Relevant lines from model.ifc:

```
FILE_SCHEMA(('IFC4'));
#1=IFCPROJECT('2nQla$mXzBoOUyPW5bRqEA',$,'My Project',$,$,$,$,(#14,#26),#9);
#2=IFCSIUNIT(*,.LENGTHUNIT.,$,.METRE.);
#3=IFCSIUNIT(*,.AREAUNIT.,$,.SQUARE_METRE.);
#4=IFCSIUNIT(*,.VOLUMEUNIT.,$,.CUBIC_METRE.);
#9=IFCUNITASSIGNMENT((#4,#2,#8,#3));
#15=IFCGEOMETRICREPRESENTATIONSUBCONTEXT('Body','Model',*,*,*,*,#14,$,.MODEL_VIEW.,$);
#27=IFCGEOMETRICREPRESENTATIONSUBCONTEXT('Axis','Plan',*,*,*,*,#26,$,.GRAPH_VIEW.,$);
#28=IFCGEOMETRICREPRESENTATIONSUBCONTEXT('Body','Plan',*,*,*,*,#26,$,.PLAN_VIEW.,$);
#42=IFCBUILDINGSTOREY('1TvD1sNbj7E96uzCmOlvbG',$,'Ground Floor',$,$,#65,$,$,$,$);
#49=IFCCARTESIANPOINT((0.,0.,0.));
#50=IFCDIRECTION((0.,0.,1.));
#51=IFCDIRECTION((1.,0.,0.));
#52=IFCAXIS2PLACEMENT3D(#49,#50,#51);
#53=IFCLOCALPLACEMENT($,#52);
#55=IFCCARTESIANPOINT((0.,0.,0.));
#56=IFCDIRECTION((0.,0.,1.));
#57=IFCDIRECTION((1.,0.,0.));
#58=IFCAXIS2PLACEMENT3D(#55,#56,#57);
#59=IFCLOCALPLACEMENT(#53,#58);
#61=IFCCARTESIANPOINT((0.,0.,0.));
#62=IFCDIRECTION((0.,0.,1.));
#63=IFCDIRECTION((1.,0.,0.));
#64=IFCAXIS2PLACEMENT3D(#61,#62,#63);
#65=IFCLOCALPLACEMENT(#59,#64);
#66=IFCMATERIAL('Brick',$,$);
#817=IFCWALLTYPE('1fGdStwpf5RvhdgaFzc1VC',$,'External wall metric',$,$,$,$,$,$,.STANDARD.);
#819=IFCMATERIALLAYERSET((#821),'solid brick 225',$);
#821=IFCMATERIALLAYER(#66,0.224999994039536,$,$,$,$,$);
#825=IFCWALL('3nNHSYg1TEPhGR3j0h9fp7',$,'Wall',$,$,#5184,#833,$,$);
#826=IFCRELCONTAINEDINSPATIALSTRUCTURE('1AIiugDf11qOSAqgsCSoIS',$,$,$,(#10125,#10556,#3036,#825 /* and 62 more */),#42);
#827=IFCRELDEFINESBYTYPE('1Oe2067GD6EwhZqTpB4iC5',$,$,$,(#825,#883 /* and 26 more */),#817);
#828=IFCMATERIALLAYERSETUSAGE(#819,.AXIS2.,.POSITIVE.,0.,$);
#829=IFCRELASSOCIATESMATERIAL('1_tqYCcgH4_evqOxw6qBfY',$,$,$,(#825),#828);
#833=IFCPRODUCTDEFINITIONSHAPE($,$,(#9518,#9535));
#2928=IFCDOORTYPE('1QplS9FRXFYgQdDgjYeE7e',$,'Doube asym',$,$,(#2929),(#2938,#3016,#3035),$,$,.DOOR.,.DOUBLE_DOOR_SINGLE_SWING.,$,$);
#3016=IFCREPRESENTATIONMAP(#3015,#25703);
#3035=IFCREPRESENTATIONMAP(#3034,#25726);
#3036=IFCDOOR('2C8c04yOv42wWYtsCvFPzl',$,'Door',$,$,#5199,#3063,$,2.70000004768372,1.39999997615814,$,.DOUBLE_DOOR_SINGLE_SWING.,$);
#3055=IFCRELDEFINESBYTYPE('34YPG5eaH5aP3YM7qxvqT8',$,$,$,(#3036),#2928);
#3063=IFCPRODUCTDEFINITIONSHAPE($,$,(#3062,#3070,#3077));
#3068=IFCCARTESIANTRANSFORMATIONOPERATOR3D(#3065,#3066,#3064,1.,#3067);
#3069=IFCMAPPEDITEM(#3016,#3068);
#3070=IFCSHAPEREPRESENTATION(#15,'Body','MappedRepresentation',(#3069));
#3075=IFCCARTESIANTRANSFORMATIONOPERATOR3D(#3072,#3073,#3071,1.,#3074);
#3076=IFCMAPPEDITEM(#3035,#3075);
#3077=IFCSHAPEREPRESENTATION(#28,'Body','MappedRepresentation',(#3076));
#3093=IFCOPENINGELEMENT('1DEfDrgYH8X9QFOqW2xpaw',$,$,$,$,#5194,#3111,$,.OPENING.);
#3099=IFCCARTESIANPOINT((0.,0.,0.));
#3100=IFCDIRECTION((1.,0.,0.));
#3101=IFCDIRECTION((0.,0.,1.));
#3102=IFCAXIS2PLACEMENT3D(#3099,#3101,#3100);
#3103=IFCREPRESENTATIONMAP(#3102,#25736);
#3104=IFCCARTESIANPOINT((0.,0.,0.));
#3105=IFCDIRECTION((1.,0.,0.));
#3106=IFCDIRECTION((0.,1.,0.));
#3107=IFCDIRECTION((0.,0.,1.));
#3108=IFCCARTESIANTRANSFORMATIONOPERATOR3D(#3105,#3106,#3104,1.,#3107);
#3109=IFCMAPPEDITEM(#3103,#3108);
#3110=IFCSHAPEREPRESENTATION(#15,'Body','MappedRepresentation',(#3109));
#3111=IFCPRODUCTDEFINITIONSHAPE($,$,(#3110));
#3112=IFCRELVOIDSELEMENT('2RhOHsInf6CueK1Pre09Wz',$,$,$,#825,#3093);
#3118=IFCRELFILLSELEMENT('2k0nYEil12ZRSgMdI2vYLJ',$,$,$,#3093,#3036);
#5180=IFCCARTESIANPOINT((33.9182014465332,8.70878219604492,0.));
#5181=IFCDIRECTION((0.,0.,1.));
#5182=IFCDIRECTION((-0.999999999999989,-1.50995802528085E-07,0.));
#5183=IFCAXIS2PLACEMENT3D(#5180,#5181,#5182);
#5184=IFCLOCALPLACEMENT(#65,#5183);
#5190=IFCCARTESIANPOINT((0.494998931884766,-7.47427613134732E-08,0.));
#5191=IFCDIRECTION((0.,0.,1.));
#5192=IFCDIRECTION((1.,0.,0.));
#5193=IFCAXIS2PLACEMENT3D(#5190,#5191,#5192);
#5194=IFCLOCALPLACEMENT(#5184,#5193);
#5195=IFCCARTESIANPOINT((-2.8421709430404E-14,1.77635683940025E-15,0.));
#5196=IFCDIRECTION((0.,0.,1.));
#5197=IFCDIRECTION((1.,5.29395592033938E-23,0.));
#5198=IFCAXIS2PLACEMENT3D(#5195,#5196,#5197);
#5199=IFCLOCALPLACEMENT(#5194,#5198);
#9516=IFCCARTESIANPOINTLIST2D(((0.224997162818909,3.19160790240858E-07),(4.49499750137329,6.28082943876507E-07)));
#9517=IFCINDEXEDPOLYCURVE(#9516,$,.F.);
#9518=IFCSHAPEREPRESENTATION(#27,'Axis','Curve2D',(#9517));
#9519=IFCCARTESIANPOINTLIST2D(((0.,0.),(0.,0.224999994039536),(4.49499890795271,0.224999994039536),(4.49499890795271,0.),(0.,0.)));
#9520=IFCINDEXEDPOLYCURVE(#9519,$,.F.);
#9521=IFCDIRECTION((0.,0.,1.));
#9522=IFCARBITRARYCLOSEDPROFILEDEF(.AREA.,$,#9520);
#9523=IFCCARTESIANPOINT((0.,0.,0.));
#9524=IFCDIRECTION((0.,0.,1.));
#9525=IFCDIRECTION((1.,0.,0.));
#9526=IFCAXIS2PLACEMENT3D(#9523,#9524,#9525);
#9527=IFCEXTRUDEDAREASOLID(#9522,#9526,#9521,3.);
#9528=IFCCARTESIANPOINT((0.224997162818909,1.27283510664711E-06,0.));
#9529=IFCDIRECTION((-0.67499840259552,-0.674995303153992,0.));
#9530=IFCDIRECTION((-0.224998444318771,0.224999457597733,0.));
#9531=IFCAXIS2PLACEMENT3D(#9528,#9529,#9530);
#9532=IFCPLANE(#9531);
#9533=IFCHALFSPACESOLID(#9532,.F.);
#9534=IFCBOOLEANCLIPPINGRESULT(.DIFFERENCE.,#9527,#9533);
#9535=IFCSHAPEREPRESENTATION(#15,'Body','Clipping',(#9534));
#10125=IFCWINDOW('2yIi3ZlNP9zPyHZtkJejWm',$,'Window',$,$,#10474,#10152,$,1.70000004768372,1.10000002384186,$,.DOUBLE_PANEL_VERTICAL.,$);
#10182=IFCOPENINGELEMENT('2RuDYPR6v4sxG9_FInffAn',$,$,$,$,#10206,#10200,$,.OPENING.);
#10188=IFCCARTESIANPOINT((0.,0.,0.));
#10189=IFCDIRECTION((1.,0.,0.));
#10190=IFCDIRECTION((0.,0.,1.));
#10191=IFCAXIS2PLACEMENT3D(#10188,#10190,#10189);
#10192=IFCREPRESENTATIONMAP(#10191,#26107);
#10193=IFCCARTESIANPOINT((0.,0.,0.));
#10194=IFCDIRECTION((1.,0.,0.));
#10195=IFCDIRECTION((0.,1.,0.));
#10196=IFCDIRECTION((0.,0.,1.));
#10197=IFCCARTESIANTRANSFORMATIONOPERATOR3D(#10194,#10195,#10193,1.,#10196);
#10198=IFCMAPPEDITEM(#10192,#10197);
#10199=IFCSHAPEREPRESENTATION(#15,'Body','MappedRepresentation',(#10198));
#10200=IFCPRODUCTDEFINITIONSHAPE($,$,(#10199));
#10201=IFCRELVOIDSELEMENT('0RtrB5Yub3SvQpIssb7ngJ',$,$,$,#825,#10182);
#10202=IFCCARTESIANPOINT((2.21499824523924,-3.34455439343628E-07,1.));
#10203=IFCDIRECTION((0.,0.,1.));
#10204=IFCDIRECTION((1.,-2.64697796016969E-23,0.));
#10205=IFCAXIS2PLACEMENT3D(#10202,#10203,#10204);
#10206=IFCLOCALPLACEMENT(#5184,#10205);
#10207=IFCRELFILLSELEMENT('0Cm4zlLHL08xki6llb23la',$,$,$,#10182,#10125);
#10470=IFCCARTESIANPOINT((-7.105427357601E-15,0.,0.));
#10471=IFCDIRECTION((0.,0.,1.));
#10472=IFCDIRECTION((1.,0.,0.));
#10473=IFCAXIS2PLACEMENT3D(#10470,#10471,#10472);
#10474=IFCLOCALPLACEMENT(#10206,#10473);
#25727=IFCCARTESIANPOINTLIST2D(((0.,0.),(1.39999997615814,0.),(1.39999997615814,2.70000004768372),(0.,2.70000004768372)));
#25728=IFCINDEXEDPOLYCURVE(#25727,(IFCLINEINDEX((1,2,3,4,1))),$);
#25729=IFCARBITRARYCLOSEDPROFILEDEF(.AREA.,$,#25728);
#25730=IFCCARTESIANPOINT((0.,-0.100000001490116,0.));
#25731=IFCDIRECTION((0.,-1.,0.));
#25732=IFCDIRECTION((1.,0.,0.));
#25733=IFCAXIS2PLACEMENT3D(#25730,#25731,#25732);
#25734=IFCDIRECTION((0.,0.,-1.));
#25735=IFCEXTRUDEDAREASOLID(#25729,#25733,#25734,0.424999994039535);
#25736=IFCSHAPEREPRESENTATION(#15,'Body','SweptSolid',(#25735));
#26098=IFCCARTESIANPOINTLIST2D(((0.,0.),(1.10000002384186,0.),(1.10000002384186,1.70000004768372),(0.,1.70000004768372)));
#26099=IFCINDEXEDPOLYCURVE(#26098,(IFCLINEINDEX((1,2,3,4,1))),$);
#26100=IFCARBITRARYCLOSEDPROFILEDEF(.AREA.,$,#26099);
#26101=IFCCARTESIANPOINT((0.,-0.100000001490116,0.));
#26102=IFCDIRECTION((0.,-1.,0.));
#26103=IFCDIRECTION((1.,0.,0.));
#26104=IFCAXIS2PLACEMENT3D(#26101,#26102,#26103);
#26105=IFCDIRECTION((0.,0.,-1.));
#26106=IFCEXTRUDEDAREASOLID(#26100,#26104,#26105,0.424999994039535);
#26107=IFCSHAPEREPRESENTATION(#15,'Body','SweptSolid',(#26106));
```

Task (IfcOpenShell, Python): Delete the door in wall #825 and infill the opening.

```python
import ifcopenshell
import ifcopenshell.api.feature
import ifcopenshell.api.root
import ifcopenshell.geom
import ifcopenshell.util.shape

model = ifcopenshell.open("model.ifc")
settings = ifcopenshell.geom.settings()


def volume(element):
    """Net volume in cubic metres, openings subtracted."""
    shape = ifcopenshell.geom.create_shape(settings, element)
    return ifcopenshell.util.shape.get_volume(shape.geometry)


door = model.by_id(3036)
opening = door.FillsVoids[0].RelatingOpeningElement
wall = opening.VoidsElements[0].RelatingBuildingElement
before = volume(wall)

ifcopenshell.api.root.remove_product(model, product=door)
ifcopenshell.api.feature.remove_feature(model, feature=opening)

after = volume(wall)

print(f"wall volume {before:.3f} -> {after:.3f} m3")

model.write("model_rev.ifc")
```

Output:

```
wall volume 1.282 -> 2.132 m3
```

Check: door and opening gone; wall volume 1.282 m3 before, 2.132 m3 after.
